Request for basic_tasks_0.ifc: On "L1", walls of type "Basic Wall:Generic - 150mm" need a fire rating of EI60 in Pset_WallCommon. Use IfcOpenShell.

First a look at what the model holds.

```python
import ifcopenshell
import ifcopenshell.util.element

model = ifcopenshell.open("basic_tasks_0.ifc")
print(model.schema)
storey = next(s for s in model.by_type("IfcBuildingStorey") if s.Name == "L1")
walls = [e for e in ifcopenshell.util.element.get_decomposition(storey) if e.is_a("IfcWall")]
seen = {}
for e in walls:
    element_type = ifcopenshell.util.element.get_type(e)
    key = (element_type.Name if element_type != e and element_type else None, ifcopenshell.util.element.get_pset(e, "Pset_WallCommon", "FireRating"))
    seen[key] = seen.get(key, 0) + 1
for (name, value), count in sorted(seen.items(), key=str):
    print(count, "x", name, "|", value)
```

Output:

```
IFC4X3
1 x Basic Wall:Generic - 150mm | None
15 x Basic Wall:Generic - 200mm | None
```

```python
import ifcopenshell
import ifcopenshell.api.pset
import ifcopenshell.util.element

model = ifcopenshell.open("basic_tasks_0.ifc")

storey = next(s for s in model.by_type("IfcBuildingStorey") if s.Name == "L1")
walls = [e for e in ifcopenshell.util.element.get_decomposition(storey) if e.is_a("IfcWall")]

count = 0
for e in walls:
    element_type = ifcopenshell.util.element.get_type(e)
    if element_type in (None, e) or element_type.Name != "Basic Wall:Generic - 150mm":
        continue
    # add_pset returns the element's existing set when there is one.
    pset = ifcopenshell.api.pset.add_pset(model, product=e, name="Pset_WallCommon")
    ifcopenshell.api.pset.edit_pset(model, pset=pset, properties={"FireRating": "EI60"})
    count += 1

print(count, "walls updated")

model.write("basic_tasks_0_edited.ifc")
```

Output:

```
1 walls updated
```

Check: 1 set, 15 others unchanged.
